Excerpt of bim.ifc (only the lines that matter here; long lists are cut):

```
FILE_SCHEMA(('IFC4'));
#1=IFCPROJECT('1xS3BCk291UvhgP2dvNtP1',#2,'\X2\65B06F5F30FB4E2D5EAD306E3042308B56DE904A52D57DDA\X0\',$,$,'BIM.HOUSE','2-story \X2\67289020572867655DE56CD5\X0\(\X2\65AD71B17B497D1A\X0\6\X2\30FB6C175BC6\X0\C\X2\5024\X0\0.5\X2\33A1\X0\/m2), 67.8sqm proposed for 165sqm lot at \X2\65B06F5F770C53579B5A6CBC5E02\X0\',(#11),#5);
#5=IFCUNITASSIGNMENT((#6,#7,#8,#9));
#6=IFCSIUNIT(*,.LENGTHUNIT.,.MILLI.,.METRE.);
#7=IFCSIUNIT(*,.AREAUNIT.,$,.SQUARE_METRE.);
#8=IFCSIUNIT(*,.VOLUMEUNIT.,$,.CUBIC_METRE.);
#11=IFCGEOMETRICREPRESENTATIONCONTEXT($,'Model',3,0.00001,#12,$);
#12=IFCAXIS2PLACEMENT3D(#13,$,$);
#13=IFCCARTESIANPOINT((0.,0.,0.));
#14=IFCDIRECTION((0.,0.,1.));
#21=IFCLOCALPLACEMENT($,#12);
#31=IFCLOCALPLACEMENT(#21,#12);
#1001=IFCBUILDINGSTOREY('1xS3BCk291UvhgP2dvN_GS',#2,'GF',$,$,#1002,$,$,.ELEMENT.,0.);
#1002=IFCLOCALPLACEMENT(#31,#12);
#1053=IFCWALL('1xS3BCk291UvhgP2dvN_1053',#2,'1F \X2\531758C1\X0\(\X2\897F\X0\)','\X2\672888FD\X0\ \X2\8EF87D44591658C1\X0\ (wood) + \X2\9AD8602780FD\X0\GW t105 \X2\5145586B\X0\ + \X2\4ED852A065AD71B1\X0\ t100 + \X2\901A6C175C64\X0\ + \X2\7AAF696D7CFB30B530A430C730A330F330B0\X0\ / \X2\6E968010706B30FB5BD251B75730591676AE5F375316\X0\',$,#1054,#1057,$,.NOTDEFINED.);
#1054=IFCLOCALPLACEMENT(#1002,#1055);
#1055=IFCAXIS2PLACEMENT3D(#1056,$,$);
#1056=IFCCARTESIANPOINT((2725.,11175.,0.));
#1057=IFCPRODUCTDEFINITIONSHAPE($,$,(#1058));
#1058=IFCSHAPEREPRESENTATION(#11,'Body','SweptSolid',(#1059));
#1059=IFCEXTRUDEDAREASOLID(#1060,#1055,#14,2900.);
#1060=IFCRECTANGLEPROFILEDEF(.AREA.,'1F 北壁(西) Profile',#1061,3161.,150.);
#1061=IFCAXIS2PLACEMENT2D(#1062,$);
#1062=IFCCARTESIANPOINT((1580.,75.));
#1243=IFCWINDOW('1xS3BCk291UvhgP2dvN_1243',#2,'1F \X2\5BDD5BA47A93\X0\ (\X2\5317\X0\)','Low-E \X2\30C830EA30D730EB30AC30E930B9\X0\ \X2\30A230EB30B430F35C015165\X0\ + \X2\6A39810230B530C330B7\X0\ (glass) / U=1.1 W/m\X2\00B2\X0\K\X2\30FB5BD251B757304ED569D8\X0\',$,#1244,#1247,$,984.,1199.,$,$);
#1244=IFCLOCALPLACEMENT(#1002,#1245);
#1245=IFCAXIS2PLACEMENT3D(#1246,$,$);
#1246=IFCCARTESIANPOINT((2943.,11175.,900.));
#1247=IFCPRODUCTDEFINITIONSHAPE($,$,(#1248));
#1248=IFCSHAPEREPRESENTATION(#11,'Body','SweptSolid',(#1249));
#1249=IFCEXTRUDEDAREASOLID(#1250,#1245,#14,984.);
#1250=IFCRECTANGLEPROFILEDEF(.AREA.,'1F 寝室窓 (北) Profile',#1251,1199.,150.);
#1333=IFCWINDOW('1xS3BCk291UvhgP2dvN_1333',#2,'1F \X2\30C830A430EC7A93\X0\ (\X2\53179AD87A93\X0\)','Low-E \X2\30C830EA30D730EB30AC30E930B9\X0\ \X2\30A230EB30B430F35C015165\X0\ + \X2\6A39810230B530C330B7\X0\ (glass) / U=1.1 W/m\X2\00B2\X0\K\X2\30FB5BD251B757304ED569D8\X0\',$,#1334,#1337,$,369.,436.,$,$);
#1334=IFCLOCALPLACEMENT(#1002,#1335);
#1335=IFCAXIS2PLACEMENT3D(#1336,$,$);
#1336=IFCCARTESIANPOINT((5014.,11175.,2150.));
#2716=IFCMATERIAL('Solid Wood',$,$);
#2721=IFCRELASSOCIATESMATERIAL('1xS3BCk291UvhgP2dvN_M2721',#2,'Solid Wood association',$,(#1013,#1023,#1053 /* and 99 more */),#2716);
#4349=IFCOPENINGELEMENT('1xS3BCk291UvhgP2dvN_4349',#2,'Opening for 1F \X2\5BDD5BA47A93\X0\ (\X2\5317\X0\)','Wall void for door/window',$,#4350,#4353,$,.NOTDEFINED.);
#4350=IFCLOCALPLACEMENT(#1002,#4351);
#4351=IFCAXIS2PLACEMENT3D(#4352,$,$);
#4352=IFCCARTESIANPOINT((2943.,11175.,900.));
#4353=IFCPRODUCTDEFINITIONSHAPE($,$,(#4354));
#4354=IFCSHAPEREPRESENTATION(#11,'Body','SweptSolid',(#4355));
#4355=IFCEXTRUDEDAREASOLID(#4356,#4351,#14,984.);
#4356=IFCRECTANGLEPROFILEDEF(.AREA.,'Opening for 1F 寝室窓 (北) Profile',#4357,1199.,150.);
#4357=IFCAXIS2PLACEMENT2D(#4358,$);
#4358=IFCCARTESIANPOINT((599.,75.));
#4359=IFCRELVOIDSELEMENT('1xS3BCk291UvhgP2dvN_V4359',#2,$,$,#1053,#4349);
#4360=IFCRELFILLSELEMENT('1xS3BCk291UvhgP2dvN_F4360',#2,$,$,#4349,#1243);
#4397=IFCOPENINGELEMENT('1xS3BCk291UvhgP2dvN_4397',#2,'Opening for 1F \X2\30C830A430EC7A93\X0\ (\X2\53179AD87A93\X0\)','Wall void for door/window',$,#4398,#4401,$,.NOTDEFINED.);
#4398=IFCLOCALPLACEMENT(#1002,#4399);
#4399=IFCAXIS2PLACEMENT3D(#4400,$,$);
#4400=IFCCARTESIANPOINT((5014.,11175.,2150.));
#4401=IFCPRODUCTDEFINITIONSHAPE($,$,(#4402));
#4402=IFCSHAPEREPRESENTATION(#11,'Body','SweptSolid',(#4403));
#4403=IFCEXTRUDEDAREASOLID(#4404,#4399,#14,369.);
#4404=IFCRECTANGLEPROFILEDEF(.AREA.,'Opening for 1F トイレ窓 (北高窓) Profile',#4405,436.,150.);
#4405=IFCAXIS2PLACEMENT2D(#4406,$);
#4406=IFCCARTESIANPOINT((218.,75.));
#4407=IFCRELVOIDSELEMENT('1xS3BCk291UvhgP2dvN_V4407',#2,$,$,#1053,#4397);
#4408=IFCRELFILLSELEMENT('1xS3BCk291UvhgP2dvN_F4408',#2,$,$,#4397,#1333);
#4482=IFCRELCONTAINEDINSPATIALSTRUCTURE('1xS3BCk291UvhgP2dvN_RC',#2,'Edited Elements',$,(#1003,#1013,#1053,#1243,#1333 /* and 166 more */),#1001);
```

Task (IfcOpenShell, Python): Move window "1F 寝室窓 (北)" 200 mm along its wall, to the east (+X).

```python
import ifcopenshell
import ifcopenshell.api.geometry
import ifcopenshell.util.placement
import ifcopenshell.util.unit

model = ifcopenshell.open("bim.ifc")
unit_scale = ifcopenshell.util.unit.calculate_unit_scale(model)

window = model.by_id(1243)
opening = window.FillsVoids[0].RelatingOpeningElement
wall = opening.VoidsElements[0].RelatingBuildingElement

wall_matrix = ifcopenshell.util.placement.get_local_placement(wall.ObjectPlacement)
shift = wall_matrix[:3, 0] * 0.2 / unit_scale
before = ifcopenshell.util.placement.get_local_placement(window.ObjectPlacement)[:3, 3].copy()

# The window is not placed relative to its opening, so move both.
for product in (opening, window):
    matrix = ifcopenshell.util.placement.get_local_placement(product.ObjectPlacement)
    matrix[:3, 3] += shift
    ifcopenshell.api.geometry.edit_object_placement(model, product=product, matrix=matrix, is_si=False)

after = ifcopenshell.util.placement.get_local_placement(window.ObjectPlacement)[:3, 3]
print("window moved by", (after - before).round(3) + 0.0)

model.write("bim-out.ifc")
```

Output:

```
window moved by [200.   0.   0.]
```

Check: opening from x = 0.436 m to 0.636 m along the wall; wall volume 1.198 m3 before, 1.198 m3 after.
